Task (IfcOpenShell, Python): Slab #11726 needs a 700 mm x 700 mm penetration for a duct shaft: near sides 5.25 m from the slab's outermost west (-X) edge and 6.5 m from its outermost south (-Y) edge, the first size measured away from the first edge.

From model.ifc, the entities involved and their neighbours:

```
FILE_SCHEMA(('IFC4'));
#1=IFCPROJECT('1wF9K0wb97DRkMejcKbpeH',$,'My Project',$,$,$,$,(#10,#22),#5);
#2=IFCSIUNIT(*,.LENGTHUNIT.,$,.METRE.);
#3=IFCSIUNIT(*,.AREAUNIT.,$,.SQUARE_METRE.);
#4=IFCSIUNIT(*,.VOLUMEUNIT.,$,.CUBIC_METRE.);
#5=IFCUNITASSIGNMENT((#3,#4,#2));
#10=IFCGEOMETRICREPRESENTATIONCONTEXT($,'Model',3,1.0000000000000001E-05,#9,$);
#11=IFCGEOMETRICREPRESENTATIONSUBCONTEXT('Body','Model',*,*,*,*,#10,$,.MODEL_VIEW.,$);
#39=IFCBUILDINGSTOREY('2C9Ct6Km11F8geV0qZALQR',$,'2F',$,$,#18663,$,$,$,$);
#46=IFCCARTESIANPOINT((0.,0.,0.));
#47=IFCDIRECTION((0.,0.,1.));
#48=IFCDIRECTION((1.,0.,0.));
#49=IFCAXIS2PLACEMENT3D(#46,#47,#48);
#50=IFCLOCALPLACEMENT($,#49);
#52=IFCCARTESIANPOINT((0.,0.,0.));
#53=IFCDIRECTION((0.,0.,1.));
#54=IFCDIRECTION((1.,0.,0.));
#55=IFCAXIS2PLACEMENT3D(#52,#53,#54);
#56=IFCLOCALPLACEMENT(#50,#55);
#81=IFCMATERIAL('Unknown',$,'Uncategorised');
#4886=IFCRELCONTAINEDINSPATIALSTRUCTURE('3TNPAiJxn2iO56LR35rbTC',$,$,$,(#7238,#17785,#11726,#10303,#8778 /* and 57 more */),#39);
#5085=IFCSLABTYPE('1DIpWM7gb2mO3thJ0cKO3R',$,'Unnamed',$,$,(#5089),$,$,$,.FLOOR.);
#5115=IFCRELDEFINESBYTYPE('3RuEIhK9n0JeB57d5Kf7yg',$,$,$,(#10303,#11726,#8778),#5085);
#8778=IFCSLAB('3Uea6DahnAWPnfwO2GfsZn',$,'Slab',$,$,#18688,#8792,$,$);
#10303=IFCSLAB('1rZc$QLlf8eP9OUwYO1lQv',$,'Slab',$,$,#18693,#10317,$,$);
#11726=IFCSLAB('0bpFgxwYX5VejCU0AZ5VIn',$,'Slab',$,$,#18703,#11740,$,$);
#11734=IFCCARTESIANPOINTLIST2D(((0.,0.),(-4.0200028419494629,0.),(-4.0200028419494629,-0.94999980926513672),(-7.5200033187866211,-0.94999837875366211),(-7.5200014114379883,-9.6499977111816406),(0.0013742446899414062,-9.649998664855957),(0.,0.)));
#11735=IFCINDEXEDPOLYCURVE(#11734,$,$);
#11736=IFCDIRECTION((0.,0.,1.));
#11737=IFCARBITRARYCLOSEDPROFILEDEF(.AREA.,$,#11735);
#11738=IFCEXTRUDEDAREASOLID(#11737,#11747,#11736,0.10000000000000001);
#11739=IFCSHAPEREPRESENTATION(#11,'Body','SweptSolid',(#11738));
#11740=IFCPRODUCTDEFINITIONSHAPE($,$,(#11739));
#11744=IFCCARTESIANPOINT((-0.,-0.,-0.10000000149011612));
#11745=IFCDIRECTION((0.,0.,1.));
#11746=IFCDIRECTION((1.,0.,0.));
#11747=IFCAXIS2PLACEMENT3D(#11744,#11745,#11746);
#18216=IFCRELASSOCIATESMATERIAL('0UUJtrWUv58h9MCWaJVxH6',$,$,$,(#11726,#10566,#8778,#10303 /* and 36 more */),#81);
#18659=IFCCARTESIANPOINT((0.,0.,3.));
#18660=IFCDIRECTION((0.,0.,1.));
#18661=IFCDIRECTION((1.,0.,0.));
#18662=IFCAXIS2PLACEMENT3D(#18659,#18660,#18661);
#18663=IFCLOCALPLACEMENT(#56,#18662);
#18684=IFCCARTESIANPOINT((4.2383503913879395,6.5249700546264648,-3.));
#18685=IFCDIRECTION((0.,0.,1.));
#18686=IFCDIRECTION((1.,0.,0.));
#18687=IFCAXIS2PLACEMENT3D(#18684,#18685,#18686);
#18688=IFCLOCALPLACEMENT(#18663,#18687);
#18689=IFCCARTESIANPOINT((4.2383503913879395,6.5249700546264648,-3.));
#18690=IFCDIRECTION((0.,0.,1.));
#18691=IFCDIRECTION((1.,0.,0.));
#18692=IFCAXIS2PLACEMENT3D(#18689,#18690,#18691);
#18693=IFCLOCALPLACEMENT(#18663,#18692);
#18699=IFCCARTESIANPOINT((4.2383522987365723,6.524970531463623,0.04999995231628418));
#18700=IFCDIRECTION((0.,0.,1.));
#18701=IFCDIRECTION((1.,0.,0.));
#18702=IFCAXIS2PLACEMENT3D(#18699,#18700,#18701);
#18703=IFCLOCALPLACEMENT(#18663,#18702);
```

```python
import numpy as np
import ifcopenshell
import ifcopenshell.api.feature
import ifcopenshell.api.geometry
import ifcopenshell.api.root
import ifcopenshell.geom
import ifcopenshell.util.placement
import ifcopenshell.util.representation
import ifcopenshell.util.shape
import ifcopenshell.util.unit

model = ifcopenshell.open("model.ifc")
unit_scale = ifcopenshell.util.unit.calculate_unit_scale(model)
settings = ifcopenshell.geom.settings()


def volume(element):
    """Net volume in cubic metres, openings subtracted."""
    shape = ifcopenshell.geom.create_shape(settings, element)
    return ifcopenshell.util.shape.get_volume(shape.geometry)


slab = model.by_guid("0bpFgxwYX5VejCU0AZ5VIn")
before = volume(slab)

# Extent in the slab's own axes, in metres. The edges named are its -X and -Y sides.
slab_shape = ifcopenshell.geom.create_shape(settings, slab)
vertices = ifcopenshell.util.shape.get_vertices(slab_shape.geometry)
x_min, y_min, bottom = vertices.min(axis=0)
top = vertices[:, 2].max()

opening = ifcopenshell.api.root.create_entity(model, ifc_class="IfcOpeningElement", name="Duct shaft opening", predefined_type="OPENING")
context = ifcopenshell.util.representation.get_context(model, "Model", "Body", "MODEL_VIEW")
width, depth = 0.7, 0.7
outline = [(0.0, 0.0), (width, 0.0), (width, depth), (0.0, depth), (0.0, 0.0)]
# Overshoot both faces by 50 mm so the cut is clean.
shape = ifcopenshell.api.geometry.add_slab_representation(
    model, context=context, depth=top - bottom + 0.1, polyline=outline
)
ifcopenshell.api.geometry.assign_representation(model, product=opening, representation=shape)

matrix = ifcopenshell.util.placement.get_local_placement(slab.ObjectPlacement)
matrix[:, 3] = matrix @ np.append(np.array([x_min + 5.25, y_min + 6.5, bottom - 0.05]) / unit_scale, 1.0)
ifcopenshell.api.geometry.edit_object_placement(model, product=opening, matrix=matrix, is_si=False)
ifcopenshell.api.feature.add_feature(model, feature=opening, element=slab)

after = volume(slab)

print(f"slab volume {before:.3f} -> {after:.3f} m3")

model.write("model_updated.ifc")
```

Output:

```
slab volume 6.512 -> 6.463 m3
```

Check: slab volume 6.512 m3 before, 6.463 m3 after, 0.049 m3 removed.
